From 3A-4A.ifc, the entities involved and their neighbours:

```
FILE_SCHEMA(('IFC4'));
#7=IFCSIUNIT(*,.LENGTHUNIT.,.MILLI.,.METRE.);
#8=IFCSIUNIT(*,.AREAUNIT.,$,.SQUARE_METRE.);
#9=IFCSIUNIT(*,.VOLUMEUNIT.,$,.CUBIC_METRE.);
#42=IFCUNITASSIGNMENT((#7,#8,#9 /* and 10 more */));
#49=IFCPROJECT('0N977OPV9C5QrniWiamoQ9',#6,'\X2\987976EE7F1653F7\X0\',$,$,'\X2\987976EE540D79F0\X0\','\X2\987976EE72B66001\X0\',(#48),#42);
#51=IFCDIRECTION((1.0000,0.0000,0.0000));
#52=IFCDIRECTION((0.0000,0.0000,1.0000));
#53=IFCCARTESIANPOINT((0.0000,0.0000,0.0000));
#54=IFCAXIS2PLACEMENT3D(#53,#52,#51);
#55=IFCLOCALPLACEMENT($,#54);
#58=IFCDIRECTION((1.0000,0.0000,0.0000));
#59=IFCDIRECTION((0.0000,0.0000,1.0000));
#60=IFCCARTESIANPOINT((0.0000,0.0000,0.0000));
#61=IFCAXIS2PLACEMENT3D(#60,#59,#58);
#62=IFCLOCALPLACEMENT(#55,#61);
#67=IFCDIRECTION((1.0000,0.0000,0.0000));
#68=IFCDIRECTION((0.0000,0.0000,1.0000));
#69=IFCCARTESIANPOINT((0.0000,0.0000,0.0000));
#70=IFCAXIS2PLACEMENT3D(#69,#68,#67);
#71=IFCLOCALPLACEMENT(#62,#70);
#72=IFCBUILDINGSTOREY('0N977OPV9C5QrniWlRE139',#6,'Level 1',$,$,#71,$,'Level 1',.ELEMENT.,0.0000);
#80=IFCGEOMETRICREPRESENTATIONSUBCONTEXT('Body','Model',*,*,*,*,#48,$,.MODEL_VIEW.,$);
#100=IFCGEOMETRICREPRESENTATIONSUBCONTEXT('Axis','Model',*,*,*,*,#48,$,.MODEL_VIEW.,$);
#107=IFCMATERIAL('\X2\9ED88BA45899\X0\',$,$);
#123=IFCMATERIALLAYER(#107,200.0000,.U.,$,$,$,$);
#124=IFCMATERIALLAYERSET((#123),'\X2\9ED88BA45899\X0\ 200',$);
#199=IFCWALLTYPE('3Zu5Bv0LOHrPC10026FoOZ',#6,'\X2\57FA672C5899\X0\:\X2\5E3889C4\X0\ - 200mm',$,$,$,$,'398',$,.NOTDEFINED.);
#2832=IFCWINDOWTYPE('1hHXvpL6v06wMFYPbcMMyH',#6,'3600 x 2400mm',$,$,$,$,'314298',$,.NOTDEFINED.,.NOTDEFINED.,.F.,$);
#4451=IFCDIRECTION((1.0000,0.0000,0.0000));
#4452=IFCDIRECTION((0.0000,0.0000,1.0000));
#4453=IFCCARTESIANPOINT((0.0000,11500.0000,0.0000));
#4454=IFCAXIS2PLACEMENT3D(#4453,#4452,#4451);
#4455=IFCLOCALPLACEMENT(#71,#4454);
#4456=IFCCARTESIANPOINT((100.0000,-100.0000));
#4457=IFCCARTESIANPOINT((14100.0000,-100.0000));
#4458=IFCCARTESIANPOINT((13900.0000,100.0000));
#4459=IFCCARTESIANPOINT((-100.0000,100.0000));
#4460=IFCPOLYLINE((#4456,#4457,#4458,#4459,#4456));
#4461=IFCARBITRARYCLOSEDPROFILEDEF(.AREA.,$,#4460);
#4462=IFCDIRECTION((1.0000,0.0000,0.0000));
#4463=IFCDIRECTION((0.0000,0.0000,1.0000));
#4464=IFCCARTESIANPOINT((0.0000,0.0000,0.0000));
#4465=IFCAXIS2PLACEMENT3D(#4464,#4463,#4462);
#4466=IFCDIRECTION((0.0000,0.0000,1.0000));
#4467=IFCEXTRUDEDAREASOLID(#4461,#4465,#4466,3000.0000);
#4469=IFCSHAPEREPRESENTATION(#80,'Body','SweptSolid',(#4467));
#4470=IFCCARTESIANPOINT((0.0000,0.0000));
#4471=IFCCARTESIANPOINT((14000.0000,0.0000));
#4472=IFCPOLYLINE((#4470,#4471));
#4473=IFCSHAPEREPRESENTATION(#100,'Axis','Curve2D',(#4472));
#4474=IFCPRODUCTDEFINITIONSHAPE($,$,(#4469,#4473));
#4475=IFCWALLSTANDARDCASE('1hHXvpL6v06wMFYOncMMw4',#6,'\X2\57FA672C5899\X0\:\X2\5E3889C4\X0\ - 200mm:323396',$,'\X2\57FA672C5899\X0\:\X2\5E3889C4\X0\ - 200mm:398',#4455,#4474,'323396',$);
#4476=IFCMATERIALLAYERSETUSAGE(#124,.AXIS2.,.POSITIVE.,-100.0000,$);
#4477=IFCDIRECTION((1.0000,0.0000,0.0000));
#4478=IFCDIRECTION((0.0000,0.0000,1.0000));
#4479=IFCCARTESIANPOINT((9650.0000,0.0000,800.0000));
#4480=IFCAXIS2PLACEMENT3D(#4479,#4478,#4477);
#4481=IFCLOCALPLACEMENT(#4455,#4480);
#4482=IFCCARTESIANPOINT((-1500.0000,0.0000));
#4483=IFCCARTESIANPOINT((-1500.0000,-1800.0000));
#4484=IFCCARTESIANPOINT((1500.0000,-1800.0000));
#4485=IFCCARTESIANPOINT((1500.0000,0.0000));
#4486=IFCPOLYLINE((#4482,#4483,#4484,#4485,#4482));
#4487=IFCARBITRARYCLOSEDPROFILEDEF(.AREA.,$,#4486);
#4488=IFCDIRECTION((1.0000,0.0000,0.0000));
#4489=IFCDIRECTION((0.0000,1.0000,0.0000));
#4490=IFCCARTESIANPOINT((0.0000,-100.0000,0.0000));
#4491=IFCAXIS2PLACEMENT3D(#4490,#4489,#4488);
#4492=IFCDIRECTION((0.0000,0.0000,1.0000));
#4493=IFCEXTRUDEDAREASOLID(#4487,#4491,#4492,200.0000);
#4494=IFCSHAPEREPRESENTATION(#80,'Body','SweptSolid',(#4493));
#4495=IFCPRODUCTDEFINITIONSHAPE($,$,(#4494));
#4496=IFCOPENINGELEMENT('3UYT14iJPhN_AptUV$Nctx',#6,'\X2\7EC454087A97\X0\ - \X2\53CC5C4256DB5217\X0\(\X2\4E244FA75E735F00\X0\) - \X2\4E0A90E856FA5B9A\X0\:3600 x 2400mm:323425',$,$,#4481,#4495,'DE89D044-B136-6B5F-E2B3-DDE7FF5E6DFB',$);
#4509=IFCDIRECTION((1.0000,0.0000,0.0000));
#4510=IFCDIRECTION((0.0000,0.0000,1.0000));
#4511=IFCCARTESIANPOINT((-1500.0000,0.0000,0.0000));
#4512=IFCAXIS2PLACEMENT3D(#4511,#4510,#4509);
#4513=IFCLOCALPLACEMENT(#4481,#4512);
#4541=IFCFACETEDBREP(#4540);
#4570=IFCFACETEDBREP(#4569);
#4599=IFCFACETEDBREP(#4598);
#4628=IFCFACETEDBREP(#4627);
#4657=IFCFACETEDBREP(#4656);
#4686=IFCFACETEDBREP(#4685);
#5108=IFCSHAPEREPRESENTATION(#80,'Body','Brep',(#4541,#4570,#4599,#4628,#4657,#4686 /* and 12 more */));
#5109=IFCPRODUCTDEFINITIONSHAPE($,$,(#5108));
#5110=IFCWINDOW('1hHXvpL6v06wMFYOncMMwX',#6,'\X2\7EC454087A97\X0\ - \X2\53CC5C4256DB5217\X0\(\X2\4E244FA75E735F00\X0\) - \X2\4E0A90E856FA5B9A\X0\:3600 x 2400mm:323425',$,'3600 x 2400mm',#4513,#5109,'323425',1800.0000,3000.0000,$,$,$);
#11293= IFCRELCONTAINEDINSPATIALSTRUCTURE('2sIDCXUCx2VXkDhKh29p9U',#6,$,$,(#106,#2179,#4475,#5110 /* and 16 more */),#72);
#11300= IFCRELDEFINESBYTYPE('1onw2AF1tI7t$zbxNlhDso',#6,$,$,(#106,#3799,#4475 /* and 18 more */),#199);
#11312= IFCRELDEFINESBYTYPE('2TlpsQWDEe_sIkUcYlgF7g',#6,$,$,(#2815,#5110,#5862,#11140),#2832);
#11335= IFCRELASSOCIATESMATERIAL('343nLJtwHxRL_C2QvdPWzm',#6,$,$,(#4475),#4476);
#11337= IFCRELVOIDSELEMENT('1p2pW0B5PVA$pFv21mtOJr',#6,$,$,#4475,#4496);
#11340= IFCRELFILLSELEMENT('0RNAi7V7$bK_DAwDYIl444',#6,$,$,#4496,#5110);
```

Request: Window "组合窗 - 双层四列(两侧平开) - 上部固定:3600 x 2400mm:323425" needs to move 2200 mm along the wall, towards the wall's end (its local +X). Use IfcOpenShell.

```python
import ifcopenshell
import ifcopenshell.api.geometry
import ifcopenshell.util.placement
import ifcopenshell.util.unit

model = ifcopenshell.open("3A-4A.ifc")
unit_scale = ifcopenshell.util.unit.calculate_unit_scale(model)

window = model.by_guid("1hHXvpL6v06wMFYOncMMwX")
opening = window.FillsVoids[0].RelatingOpeningElement
wall = opening.VoidsElements[0].RelatingBuildingElement

wall_matrix = ifcopenshell.util.placement.get_local_placement(wall.ObjectPlacement)
shift = wall_matrix[:3, 0] * 2.2 / unit_scale
before = ifcopenshell.util.placement.get_local_placement(window.ObjectPlacement)[:3, 3].copy()

# The window is placed relative to its opening, so it follows when the opening moves.
matrix = ifcopenshell.util.placement.get_local_placement(opening.ObjectPlacement)
matrix[:3, 3] += shift
ifcopenshell.api.geometry.edit_object_placement(
    model, product=opening, matrix=matrix, is_si=False, should_transform_children=True
)

after = ifcopenshell.util.placement.get_local_placement(window.ObjectPlacement)[:3, 3]
print("window moved by", (after - before).round(3) + 0.0)

model.write("3A-4A-out.ifc")
```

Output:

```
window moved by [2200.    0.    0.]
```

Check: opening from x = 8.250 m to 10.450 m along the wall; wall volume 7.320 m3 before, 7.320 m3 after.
